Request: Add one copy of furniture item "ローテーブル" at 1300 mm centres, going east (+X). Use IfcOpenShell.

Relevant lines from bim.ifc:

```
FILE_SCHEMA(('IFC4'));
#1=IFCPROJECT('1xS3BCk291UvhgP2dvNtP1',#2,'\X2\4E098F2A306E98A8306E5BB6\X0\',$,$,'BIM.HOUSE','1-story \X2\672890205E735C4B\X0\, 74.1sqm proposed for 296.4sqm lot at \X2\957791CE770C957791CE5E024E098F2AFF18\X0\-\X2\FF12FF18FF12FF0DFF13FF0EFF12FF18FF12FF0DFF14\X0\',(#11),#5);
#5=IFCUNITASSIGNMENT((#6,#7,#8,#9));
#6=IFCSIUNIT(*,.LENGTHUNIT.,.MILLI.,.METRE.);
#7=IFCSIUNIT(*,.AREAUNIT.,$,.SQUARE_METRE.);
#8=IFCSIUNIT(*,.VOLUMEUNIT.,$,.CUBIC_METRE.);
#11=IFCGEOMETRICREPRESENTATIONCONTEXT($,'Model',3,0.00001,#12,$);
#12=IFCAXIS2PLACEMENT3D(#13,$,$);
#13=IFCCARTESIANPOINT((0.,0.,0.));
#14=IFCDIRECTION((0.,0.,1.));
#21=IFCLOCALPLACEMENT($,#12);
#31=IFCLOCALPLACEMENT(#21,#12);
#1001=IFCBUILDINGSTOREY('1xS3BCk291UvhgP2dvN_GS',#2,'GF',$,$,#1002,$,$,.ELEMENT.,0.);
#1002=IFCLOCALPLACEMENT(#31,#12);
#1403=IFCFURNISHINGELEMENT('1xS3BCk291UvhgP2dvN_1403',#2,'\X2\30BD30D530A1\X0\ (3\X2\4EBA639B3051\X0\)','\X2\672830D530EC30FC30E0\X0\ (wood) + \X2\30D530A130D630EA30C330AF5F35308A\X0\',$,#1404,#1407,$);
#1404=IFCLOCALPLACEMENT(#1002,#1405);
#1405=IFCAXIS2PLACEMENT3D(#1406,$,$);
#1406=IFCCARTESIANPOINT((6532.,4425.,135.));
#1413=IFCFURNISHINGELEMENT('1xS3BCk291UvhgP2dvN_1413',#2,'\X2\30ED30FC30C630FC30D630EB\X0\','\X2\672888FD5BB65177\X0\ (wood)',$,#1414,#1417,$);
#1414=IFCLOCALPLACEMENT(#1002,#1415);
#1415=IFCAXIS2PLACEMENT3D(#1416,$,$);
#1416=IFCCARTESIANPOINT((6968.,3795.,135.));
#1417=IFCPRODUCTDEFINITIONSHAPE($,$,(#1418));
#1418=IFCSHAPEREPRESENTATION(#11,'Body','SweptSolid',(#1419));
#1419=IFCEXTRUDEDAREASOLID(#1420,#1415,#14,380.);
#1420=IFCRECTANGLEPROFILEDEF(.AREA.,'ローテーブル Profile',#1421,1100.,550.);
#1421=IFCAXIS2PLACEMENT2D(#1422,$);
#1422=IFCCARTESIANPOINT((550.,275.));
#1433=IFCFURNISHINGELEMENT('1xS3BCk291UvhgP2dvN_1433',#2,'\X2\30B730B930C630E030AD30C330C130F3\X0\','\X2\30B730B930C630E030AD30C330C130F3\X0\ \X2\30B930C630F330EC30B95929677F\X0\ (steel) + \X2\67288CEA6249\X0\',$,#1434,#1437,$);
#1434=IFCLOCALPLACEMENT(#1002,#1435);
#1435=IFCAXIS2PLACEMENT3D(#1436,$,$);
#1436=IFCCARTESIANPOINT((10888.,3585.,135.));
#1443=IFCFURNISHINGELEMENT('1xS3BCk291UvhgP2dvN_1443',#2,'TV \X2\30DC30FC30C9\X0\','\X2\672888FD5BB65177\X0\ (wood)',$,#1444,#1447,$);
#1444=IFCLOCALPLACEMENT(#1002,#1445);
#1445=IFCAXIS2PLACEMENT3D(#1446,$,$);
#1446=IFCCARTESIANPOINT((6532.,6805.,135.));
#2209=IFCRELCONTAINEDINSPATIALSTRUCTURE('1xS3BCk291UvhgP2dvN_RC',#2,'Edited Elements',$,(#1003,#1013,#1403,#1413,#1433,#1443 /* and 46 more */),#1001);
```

```python
import numpy as np
import ifcopenshell
import ifcopenshell.api.geometry
import ifcopenshell.api.root
import ifcopenshell.util.element
import ifcopenshell.util.placement

model = ifcopenshell.open("bim.ifc")


def reuse_history(source, copy):
    """copy_class also copies each property set's owner history, people and application; keep the originals."""
    for rel in copy.IsDefinedBy:
        if rel.is_a("IfcRelDefinesByProperties") and (history := rel.RelatingPropertyDefinition.OwnerHistory):
            rel.RelatingPropertyDefinition.OwnerHistory = source.OwnerHistory
            ifcopenshell.util.element.remove_deep2(model, history)


source = model.by_guid("1xS3BCk291UvhgP2dvN_1413")
base = ifcopenshell.util.placement.get_local_placement(source.ObjectPlacement)
step = np.array([1.0, 0.0, 0.0]) * 1300.0

for i in range(1, 2):
    copy = ifcopenshell.api.root.copy_class(model, product=source)
    copy.Representation = ifcopenshell.util.element.copy_deep(
        model, source.Representation, exclude=["IfcGeometricRepresentationContext", "IfcRepresentationMap"]
    )
    reuse_history(source, copy)
    matrix = base.copy()
    matrix[:3, 3] += i * step
    print("added at", matrix[:3, 3].round(3) + 0.0)
    ifcopenshell.api.geometry.edit_object_placement(model, product=copy, matrix=matrix, is_si=False)

model.write("bim_edited.ifc")
```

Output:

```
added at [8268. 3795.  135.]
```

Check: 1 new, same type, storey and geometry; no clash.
